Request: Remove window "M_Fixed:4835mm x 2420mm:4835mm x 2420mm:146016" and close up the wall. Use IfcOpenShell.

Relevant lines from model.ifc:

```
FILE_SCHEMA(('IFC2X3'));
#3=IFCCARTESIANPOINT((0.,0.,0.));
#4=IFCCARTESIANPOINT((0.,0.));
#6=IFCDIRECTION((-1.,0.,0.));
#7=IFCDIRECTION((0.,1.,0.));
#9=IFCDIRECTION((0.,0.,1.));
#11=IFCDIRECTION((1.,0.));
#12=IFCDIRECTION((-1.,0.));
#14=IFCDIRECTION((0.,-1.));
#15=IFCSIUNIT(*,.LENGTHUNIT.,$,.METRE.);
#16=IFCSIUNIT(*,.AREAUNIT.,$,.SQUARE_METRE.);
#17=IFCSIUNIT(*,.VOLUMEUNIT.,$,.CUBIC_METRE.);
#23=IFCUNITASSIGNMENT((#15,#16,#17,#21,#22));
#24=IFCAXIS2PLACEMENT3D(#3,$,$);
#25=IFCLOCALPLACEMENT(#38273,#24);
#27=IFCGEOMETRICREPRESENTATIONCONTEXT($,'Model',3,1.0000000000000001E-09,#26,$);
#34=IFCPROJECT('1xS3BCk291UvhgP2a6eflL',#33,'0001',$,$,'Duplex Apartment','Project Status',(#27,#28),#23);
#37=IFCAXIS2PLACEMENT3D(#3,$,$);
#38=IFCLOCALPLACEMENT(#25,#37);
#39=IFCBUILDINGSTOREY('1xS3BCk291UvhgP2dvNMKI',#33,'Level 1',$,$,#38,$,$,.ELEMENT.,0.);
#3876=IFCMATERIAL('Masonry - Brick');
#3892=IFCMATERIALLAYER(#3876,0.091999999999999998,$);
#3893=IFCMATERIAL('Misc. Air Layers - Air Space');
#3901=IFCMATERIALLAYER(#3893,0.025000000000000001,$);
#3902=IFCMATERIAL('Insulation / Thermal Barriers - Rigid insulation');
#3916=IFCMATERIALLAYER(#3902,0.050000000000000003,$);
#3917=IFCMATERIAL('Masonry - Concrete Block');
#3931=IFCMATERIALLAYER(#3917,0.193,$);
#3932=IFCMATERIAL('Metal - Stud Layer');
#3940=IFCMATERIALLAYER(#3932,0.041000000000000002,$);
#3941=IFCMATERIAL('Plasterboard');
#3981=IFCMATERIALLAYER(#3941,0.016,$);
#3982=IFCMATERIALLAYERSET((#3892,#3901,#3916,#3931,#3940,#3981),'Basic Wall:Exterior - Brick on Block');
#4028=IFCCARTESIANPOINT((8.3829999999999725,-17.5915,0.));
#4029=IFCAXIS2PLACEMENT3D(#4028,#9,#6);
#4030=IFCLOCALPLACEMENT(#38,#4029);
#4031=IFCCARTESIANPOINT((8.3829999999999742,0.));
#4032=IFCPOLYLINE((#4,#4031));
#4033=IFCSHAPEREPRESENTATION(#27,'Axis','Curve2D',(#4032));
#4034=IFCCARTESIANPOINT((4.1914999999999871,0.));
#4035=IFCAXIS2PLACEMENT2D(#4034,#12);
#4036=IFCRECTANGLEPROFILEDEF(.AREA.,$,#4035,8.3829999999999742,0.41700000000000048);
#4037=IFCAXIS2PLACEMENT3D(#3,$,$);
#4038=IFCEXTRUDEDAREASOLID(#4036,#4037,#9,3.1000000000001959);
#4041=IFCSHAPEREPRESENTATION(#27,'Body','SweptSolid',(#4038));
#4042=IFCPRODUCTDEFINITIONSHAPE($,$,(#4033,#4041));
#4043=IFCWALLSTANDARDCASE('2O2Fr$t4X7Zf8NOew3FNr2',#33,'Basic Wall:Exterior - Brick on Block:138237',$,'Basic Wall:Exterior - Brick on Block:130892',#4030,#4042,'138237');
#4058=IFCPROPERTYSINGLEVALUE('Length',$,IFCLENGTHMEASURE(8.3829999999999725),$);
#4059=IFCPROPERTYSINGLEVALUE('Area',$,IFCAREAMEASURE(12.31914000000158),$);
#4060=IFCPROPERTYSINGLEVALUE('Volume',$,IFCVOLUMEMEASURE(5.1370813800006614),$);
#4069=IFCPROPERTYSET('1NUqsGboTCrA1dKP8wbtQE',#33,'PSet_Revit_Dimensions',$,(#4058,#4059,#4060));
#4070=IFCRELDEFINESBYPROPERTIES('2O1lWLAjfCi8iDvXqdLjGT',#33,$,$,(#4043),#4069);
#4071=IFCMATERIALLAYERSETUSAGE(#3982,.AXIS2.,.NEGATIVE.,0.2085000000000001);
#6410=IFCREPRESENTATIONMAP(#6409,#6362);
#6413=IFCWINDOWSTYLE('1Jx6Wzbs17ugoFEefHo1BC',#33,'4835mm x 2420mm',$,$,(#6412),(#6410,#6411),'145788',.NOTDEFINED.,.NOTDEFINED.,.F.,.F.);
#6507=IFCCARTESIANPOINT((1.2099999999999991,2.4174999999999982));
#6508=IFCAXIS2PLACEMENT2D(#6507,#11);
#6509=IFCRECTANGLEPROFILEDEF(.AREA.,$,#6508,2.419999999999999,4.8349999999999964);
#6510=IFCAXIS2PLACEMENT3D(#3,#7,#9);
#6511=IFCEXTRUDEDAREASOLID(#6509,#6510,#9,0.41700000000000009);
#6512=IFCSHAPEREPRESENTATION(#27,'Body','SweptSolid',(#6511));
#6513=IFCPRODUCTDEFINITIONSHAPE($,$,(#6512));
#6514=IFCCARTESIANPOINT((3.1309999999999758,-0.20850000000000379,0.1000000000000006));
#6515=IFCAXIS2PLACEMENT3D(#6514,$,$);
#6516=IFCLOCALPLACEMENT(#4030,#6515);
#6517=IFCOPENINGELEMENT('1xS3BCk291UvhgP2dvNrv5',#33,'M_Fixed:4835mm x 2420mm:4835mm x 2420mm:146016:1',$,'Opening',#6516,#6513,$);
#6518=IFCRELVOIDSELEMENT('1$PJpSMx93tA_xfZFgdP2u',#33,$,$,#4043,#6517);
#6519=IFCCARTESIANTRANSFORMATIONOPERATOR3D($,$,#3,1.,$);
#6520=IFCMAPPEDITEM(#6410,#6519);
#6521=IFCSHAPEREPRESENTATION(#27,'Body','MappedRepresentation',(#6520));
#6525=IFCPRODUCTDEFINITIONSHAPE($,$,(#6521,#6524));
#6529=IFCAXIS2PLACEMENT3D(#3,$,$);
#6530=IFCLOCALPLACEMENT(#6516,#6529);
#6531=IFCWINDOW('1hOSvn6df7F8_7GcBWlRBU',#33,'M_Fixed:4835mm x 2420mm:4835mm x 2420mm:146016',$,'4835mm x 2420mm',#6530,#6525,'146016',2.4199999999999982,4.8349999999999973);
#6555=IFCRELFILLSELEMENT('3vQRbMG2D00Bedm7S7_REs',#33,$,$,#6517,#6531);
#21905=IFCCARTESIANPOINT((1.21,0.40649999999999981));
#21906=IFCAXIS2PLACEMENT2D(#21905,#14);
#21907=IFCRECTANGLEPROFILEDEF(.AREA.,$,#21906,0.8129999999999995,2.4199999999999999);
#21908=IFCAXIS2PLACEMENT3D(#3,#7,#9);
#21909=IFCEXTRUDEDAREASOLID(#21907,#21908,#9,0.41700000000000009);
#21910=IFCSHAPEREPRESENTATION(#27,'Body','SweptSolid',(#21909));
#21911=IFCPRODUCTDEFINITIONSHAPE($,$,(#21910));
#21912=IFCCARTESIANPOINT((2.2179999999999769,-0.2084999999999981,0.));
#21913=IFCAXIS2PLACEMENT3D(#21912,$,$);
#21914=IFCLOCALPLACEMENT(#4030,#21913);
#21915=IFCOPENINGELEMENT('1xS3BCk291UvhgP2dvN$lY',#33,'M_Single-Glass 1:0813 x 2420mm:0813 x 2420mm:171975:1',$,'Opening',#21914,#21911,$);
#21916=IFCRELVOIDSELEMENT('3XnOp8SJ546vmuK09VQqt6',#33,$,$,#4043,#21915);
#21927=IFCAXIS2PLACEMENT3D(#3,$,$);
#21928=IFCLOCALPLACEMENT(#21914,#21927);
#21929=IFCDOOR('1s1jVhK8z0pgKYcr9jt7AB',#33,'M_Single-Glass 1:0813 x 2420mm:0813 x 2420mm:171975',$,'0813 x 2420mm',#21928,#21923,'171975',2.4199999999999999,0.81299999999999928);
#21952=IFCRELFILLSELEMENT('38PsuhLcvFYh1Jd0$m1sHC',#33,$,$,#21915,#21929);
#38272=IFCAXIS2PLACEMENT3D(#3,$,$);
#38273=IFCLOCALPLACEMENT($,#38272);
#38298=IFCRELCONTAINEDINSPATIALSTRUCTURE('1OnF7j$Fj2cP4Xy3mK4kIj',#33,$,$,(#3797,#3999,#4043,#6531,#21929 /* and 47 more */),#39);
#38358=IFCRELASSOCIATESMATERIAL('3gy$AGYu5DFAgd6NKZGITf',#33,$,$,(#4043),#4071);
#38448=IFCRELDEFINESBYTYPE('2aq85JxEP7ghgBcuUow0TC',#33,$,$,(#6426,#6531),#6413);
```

```python
import ifcopenshell
import ifcopenshell.api.feature
import ifcopenshell.api.pset
import ifcopenshell.api.root
import ifcopenshell.geom
import ifcopenshell.util.element
import ifcopenshell.util.shape
import ifcopenshell.util.unit

model = ifcopenshell.open("model.ifc")
area_scale = ifcopenshell.util.unit.calculate_unit_scale(model, "AREAUNIT")
volume_scale = ifcopenshell.util.unit.calculate_unit_scale(model, "VOLUMEUNIT")
settings = ifcopenshell.geom.settings()


def volume(element):
    """Net volume in cubic metres, openings subtracted."""
    shape = ifcopenshell.geom.create_shape(settings, element)
    return ifcopenshell.util.shape.get_volume(shape.geometry)


window = model.by_guid("1hOSvn6df7F8_7GcBWlRBU")
opening = window.FillsVoids[0].RelatingOpeningElement
wall = opening.VoidsElements[0].RelatingBuildingElement
before = volume(wall)

ifcopenshell.api.root.remove_product(model, product=window)
ifcopenshell.api.feature.remove_feature(model, feature=opening)

after = volume(wall)
thickness = 0.417  # wall thickness in metres

# Update the wall's stored quantities.
pset = model.by_id(ifcopenshell.util.element.get_pset(wall, "PSet_Revit_Dimensions", should_inherit=False)["id"])
ifcopenshell.api.pset.edit_pset(model, pset=pset, properties={
    "Area": model.create_entity("IfcAreaMeasure", after / thickness / area_scale),
    "Volume": model.create_entity("IfcVolumeMeasure", after / volume_scale),
})

print(f"wall volume {before:.3f} -> {after:.3f} m3")

model.write("model_v2.ifc")
```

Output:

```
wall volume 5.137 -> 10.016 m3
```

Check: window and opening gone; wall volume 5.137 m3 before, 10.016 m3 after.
